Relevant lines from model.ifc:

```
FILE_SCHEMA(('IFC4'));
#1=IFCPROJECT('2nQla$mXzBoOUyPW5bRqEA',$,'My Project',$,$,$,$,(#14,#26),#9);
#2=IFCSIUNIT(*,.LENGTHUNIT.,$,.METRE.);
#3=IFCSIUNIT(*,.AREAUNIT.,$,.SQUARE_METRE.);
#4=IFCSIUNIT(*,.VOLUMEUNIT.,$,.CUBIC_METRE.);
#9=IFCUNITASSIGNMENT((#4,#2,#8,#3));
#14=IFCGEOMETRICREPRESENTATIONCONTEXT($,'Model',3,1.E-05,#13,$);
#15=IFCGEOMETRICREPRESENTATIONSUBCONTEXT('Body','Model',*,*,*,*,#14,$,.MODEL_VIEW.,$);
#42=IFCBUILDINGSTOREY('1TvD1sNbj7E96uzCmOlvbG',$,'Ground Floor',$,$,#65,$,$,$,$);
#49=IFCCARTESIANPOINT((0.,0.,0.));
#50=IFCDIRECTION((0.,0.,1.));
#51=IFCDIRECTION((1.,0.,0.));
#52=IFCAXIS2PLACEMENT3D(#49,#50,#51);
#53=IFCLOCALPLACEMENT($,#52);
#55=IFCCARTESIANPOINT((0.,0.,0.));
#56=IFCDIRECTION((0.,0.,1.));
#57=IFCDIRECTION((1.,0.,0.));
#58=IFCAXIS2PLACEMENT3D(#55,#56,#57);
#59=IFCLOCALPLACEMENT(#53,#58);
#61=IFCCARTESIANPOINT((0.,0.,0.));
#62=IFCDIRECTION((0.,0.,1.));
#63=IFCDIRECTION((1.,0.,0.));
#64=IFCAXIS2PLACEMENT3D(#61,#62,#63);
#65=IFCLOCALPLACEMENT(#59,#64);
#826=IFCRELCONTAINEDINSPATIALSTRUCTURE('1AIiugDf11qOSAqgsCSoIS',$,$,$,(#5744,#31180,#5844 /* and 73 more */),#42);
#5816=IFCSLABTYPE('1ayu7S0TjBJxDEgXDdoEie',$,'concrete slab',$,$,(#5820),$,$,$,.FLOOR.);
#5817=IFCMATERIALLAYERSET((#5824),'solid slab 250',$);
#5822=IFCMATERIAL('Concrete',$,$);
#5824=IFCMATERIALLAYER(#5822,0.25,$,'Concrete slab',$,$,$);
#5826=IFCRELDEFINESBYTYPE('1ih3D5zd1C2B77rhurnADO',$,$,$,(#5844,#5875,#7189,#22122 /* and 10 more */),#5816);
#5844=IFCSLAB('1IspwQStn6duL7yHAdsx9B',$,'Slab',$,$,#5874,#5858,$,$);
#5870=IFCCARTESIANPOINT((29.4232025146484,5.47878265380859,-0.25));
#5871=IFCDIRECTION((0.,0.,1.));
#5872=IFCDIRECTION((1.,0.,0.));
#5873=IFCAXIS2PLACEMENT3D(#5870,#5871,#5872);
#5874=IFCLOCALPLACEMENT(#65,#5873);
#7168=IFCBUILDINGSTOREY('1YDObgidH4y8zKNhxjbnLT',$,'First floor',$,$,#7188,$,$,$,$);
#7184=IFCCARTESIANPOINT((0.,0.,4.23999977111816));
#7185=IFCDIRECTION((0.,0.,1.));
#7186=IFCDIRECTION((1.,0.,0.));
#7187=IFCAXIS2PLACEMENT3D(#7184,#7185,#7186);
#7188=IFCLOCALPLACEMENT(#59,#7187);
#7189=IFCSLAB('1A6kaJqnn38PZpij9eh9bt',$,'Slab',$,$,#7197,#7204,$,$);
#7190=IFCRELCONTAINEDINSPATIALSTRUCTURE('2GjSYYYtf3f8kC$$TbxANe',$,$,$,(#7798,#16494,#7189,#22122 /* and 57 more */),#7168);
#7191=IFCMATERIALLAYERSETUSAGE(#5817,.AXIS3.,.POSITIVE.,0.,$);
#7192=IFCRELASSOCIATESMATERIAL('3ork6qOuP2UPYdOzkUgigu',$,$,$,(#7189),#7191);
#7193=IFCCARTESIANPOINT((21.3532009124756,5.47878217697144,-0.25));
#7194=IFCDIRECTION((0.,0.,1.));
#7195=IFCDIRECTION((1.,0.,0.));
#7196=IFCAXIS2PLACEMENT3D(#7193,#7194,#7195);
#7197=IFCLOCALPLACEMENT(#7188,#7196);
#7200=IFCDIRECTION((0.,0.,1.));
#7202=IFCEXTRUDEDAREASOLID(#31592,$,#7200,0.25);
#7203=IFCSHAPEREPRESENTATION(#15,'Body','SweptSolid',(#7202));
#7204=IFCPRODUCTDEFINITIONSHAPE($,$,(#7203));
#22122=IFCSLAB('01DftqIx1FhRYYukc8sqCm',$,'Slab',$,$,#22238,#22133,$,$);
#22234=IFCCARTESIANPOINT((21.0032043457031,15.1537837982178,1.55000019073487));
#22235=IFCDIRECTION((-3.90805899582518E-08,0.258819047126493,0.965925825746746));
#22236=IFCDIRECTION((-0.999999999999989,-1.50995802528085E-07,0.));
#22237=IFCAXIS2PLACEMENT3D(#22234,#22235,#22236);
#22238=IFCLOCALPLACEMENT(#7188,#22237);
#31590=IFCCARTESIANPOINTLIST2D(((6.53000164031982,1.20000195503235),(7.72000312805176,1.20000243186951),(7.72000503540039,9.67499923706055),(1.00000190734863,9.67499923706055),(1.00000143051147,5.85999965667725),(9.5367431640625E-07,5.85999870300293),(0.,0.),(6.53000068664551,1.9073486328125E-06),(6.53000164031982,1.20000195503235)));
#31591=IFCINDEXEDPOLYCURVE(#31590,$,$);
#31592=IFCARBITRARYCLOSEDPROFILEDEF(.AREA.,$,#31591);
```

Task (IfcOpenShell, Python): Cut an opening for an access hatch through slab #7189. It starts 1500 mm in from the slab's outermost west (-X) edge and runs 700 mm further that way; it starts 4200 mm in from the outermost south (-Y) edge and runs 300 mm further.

```python
import numpy as np
import ifcopenshell
import ifcopenshell.api.feature
import ifcopenshell.api.geometry
import ifcopenshell.api.root
import ifcopenshell.geom
import ifcopenshell.util.placement
import ifcopenshell.util.representation
import ifcopenshell.util.shape
import ifcopenshell.util.unit

model = ifcopenshell.open("model.ifc")
unit_scale = ifcopenshell.util.unit.calculate_unit_scale(model)
settings = ifcopenshell.geom.settings()


def volume(element):
    """Net volume in cubic metres, openings subtracted."""
    shape = ifcopenshell.geom.create_shape(settings, element)
    return ifcopenshell.util.shape.get_volume(shape.geometry)


slab = model.by_guid("1A6kaJqnn38PZpij9eh9bt")
before = volume(slab)

# Extent in the slab's own axes, in metres. The edges named are its -X and -Y sides.
slab_shape = ifcopenshell.geom.create_shape(settings, slab)
vertices = ifcopenshell.util.shape.get_vertices(slab_shape.geometry)
x_min, y_min, bottom = vertices.min(axis=0)
top = vertices[:, 2].max()

opening = ifcopenshell.api.root.create_entity(model, ifc_class="IfcOpeningElement", name="Access hatch opening", predefined_type="OPENING")
context = ifcopenshell.util.representation.get_context(model, "Model", "Body", "MODEL_VIEW")
width, depth = 0.7, 0.3
outline = [(0.0, 0.0), (width, 0.0), (width, depth), (0.0, depth), (0.0, 0.0)]
# Overshoot both faces by 50 mm so the cut is clean.
shape = ifcopenshell.api.geometry.add_slab_representation(
    model, context=context, depth=top - bottom + 0.1, polyline=outline
)
ifcopenshell.api.geometry.assign_representation(model, product=opening, representation=shape)

matrix = ifcopenshell.util.placement.get_local_placement(slab.ObjectPlacement)
matrix[:, 3] = matrix @ np.append(np.array([x_min + 1.5, y_min + 4.2, bottom - 0.05]) / unit_scale, 1.0)
ifcopenshell.api.geometry.edit_object_placement(model, product=opening, matrix=matrix, is_si=False)
ifcopenshell.api.feature.add_feature(model, feature=opening, element=slab)

after = volume(slab)

print(f"slab volume {before:.3f} -> {after:.3f} m3")

model.write("model_edited.ifc")
```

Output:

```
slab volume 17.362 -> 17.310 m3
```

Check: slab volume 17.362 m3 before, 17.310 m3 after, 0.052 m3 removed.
